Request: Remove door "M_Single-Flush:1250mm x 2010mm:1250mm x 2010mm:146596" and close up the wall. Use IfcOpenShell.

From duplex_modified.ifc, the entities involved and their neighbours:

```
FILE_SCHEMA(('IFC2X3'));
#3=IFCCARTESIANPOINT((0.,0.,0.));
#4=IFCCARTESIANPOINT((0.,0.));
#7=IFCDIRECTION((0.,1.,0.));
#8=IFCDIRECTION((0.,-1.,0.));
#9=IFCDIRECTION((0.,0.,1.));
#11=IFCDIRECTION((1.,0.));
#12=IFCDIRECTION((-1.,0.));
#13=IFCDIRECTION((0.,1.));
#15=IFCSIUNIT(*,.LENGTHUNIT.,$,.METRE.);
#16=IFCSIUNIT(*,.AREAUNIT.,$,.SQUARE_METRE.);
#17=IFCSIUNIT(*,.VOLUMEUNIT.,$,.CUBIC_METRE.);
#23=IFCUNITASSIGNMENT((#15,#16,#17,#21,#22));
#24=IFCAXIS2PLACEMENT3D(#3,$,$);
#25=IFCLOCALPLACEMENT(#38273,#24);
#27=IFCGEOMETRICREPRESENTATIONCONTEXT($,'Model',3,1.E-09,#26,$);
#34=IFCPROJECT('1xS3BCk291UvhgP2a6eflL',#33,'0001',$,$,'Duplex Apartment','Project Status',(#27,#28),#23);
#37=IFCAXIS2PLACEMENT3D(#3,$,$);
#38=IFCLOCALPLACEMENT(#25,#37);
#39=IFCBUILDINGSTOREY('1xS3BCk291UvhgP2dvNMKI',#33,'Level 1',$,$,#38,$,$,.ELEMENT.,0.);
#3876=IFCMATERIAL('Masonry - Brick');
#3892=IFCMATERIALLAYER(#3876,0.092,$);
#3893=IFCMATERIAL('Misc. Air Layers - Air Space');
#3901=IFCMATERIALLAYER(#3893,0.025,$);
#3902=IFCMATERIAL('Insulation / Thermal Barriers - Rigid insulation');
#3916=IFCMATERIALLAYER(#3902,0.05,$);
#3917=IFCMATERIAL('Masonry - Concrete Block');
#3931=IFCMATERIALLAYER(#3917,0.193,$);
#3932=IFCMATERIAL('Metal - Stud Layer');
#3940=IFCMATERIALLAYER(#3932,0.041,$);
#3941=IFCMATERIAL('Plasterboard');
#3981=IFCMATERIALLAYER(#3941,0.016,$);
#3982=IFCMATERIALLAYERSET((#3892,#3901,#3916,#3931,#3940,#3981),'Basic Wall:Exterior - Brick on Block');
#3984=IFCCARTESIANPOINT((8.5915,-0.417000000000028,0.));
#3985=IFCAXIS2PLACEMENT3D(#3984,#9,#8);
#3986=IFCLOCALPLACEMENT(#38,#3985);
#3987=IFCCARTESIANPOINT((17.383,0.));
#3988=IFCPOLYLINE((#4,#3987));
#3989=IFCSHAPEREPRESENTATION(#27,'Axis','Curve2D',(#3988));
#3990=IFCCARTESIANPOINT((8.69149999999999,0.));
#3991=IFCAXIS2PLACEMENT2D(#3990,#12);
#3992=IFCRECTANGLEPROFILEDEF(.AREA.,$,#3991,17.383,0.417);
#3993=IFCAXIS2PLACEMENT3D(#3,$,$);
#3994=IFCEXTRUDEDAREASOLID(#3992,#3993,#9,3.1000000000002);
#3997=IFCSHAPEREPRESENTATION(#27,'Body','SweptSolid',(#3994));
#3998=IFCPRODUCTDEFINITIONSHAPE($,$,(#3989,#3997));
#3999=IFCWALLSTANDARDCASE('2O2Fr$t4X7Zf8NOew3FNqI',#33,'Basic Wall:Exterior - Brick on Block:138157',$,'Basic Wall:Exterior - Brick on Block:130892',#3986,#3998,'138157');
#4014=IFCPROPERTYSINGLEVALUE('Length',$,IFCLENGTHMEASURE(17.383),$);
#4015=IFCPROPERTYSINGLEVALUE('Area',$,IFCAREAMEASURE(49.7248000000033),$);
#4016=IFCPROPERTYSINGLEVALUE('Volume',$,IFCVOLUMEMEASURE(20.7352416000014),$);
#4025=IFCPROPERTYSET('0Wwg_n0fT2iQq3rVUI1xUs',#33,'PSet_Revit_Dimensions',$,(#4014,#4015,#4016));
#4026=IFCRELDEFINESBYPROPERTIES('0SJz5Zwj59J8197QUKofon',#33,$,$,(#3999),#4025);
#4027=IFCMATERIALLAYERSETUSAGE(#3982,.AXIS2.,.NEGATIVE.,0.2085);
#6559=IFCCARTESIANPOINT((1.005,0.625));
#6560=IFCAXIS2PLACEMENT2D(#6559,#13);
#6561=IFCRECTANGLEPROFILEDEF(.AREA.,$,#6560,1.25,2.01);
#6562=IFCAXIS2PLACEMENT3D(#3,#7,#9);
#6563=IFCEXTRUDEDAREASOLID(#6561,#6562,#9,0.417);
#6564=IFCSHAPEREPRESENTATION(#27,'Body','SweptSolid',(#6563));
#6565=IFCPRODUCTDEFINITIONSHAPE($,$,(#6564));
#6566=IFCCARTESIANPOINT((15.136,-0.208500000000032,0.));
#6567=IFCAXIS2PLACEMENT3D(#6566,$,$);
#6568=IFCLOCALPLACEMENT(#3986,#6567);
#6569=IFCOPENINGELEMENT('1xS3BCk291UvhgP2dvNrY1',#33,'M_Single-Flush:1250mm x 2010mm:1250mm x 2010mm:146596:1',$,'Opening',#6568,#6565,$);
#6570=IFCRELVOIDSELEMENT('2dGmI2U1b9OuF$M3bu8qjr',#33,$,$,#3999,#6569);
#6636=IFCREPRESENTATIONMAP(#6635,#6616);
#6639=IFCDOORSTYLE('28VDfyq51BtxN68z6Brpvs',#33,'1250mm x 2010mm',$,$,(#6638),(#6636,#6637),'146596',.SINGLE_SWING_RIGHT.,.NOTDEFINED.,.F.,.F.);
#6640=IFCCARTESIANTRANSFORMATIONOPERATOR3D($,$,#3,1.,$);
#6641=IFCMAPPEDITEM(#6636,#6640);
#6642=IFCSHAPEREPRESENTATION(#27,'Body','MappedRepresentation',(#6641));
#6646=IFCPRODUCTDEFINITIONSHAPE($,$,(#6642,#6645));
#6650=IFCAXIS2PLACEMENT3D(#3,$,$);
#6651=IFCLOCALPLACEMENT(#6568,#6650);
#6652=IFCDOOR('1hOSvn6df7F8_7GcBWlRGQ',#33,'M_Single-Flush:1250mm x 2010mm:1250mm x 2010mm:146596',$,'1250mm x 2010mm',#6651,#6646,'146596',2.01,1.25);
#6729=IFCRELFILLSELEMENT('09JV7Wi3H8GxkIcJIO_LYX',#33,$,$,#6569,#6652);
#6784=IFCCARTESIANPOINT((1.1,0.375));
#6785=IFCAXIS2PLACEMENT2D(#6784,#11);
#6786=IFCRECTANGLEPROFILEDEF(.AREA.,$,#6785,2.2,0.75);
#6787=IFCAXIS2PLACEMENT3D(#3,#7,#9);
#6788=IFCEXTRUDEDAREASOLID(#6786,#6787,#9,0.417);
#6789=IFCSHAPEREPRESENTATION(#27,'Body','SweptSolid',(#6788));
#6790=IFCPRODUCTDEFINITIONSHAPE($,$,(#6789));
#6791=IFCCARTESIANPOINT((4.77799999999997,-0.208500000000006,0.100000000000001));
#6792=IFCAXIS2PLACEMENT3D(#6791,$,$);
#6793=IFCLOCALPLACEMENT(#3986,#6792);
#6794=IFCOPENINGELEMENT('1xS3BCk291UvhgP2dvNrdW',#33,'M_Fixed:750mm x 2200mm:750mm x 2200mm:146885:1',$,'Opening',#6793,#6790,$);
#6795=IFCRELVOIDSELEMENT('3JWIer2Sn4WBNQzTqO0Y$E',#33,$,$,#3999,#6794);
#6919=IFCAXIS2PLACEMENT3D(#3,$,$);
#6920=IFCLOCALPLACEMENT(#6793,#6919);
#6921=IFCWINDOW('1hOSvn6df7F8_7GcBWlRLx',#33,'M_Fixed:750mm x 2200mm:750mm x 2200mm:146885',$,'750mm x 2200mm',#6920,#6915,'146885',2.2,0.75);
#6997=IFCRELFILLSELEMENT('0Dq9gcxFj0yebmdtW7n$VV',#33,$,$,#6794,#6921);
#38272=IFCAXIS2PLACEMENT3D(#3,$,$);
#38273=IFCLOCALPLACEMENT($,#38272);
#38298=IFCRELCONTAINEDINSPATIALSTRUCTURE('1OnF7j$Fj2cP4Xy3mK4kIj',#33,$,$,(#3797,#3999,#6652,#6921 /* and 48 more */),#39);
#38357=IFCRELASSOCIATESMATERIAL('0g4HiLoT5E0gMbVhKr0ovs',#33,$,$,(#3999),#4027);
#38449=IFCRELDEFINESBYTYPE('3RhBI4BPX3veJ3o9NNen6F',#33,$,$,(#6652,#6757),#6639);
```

```python
import ifcopenshell
import ifcopenshell.api.feature
import ifcopenshell.api.pset
import ifcopenshell.api.root
import ifcopenshell.geom
import ifcopenshell.util.element
import ifcopenshell.util.shape
import ifcopenshell.util.unit

model = ifcopenshell.open("duplex_modified.ifc")
area_scale = ifcopenshell.util.unit.calculate_unit_scale(model, "AREAUNIT")
volume_scale = ifcopenshell.util.unit.calculate_unit_scale(model, "VOLUMEUNIT")
settings = ifcopenshell.geom.settings()


def volume(element):
    """Net volume in cubic metres, openings subtracted."""
    shape = ifcopenshell.geom.create_shape(settings, element)
    return ifcopenshell.util.shape.get_volume(shape.geometry)


door = model.by_guid("1hOSvn6df7F8_7GcBWlRGQ")
opening = door.FillsVoids[0].RelatingOpeningElement
wall = opening.VoidsElements[0].RelatingBuildingElement
before = volume(wall)

ifcopenshell.api.root.remove_product(model, product=door)
ifcopenshell.api.feature.remove_feature(model, feature=opening)

after = volume(wall)
thickness = 0.417  # wall thickness in metres

# Update the wall's stored quantities.
pset = model.by_id(ifcopenshell.util.element.get_pset(wall, "PSet_Revit_Dimensions", should_inherit=False)["id"])
ifcopenshell.api.pset.edit_pset(model, pset=pset, properties={
    "Area": model.create_entity("IfcAreaMeasure", after / thickness / area_scale),
    "Volume": model.create_entity("IfcVolumeMeasure", after / volume_scale),
})

print(f"wall volume {before:.3f} -> {after:.3f} m3")

model.write("duplex_modified_v2.ifc")
```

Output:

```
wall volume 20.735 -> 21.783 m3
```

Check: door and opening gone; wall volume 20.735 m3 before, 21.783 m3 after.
